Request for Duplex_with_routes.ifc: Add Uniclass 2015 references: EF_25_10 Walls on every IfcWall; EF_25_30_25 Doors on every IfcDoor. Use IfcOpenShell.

First a look at what the model holds.

```python
import ifcopenshell

model = ifcopenshell.open("Duplex_with_routes.ifc")
print(model.schema)
print("classifications:", [c.Name for c in model.by_type("IfcClassification")])
for ifc_class in ("IfcDoor", "IfcRoof", "IfcStair", "IfcWall", "IfcWindow"):
    print(ifc_class, len(model.by_type(ifc_class)))
```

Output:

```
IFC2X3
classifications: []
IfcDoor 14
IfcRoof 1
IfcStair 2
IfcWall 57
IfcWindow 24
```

```python
import ifcopenshell
import ifcopenshell.api.classification

model = ifcopenshell.open("Duplex_with_routes.ifc")

# IFC2X3 requires Source and Edition and has no link from the project to the system.
system = model.create_entity("IfcClassification", Source="NBS", Edition="2015", Name="Uniclass 2015")

codes = {
    "IfcWall": ("EF_25_10", "Walls"),
    "IfcDoor": ("EF_25_30_25", "Doors"),
}
for ifc_class, (code, name) in codes.items():
    products = model.by_type(ifc_class)
    ifcopenshell.api.classification.add_reference(
        model, products=products, classification=system, identification=code, name=name
    )
    print(code, len(products))

model.write("Duplex_with_routes_updated.ifc")
```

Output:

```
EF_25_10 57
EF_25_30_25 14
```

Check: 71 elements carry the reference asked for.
